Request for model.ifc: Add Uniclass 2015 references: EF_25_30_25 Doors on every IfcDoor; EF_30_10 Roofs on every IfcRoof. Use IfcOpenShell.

First a look at what the model holds.

```python
import ifcopenshell

model = ifcopenshell.open("model.ifc")
print(model.schema)
print("classifications:", [c.Name for c in model.by_type("IfcClassification")])
for ifc_class in ("IfcDoor", "IfcRoof", "IfcStair", "IfcWall", "IfcWindow"):
    print(ifc_class, len(model.by_type(ifc_class)))
```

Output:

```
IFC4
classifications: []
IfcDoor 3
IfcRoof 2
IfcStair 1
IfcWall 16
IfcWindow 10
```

```python
import ifcopenshell
import ifcopenshell.api.classification

model = ifcopenshell.open("model.ifc")

system = ifcopenshell.api.classification.add_classification(model, classification="Uniclass 2015")

codes = {
    "IfcDoor": ("EF_25_30_25", "Doors"),
    "IfcRoof": ("EF_30_10", "Roofs"),
}
for ifc_class, (code, name) in codes.items():
    products = model.by_type(ifc_class)
    ifcopenshell.api.classification.add_reference(
        model, products=products, classification=system, identification=code, name=name
    )
    print(code, len(products))

model.write("model_rev.ifc")
```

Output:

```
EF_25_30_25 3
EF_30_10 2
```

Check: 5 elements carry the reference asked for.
